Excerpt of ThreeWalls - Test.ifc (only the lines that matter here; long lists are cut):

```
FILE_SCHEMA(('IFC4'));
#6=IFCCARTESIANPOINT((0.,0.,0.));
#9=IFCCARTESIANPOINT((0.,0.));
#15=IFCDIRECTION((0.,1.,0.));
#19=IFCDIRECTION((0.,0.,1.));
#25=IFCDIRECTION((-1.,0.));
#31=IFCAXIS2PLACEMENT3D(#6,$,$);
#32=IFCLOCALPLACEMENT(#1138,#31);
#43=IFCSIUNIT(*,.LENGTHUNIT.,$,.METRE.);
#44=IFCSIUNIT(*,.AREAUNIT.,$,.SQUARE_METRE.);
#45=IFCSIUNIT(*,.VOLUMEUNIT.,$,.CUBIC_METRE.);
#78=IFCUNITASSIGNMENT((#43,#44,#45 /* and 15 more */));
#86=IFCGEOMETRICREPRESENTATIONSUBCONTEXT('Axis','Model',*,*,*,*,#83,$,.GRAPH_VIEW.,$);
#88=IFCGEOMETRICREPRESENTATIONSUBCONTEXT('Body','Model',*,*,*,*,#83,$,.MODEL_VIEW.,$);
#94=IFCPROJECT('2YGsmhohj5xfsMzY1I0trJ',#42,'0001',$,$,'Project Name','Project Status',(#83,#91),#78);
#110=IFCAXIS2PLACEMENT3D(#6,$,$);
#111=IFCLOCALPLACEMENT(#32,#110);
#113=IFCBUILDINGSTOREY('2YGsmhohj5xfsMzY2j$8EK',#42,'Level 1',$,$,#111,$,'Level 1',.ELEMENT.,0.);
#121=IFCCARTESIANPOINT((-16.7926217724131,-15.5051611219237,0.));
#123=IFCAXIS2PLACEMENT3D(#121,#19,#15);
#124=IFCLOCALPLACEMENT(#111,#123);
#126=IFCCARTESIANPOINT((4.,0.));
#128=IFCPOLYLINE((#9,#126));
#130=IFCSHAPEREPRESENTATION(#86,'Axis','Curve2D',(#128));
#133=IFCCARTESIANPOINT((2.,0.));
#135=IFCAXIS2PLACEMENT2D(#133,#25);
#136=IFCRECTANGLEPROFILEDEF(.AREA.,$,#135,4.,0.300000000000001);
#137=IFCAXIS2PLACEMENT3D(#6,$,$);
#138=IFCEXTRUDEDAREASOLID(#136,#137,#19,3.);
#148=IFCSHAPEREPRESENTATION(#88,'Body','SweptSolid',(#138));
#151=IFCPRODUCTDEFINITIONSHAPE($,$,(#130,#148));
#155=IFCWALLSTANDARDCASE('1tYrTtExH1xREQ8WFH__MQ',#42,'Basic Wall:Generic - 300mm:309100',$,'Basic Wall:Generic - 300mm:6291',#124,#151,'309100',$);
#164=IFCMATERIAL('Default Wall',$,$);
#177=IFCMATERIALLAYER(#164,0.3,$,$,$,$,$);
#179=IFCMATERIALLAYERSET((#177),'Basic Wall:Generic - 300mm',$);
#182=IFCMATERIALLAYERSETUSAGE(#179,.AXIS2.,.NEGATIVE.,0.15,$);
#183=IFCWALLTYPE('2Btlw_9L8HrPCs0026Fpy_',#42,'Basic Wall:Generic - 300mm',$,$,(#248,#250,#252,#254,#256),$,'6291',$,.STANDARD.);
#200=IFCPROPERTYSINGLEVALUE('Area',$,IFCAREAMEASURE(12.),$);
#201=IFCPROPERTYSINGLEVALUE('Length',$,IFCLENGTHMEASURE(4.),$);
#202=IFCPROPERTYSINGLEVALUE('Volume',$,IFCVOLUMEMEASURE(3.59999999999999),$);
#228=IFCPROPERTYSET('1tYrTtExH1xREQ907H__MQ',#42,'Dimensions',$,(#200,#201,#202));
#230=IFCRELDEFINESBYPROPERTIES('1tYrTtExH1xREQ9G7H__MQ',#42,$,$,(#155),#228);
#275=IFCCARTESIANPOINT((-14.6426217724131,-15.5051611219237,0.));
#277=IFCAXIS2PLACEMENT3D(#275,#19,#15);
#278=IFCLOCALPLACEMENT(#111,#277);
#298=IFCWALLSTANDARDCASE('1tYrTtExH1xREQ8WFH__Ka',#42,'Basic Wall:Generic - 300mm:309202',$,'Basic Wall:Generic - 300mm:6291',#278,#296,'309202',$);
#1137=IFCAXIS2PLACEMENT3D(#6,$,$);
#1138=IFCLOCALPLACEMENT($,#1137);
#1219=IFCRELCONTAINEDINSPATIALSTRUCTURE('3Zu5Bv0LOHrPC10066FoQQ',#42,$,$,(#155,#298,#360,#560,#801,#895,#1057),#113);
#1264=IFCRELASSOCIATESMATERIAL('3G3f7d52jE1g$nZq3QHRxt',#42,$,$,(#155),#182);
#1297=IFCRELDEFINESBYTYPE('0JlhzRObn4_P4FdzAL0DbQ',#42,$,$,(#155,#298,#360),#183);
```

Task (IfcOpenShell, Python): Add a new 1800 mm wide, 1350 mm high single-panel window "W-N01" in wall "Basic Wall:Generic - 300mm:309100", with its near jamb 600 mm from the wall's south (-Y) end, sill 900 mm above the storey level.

```python
import numpy as np
import ifcopenshell
import ifcopenshell.api.feature
import ifcopenshell.api.geometry
import ifcopenshell.api.pset
import ifcopenshell.api.root
import ifcopenshell.api.spatial
import ifcopenshell.geom
import ifcopenshell.util.element
import ifcopenshell.util.placement
import ifcopenshell.util.representation
import ifcopenshell.util.shape
import ifcopenshell.util.unit

model = ifcopenshell.open("ThreeWalls - Test.ifc")
unit_scale = ifcopenshell.util.unit.calculate_unit_scale(model)
area_scale = ifcopenshell.util.unit.calculate_unit_scale(model, "AREAUNIT")
volume_scale = ifcopenshell.util.unit.calculate_unit_scale(model, "VOLUMEUNIT")
settings = ifcopenshell.geom.settings()


def volume(element):
    """Net volume in cubic metres, openings subtracted."""
    shape = ifcopenshell.geom.create_shape(settings, element)
    return ifcopenshell.util.shape.get_volume(shape.geometry)


wall = model.by_guid("1tYrTtExH1xREQ8WFH__MQ")
storey = ifcopenshell.util.element.get_container(wall, ifc_class="IfcBuildingStorey")
context = ifcopenshell.util.representation.get_context(model, "Model", "Body", "MODEL_VIEW")
before = volume(wall)

width, height, from_end, sill = 1.8, 1.35, 0.6, 0.9  # metres

# The wall runs along its own X axis, and the end named is its -X end.
wall_shape = ifcopenshell.geom.create_shape(settings, wall)
x, y, z = ifcopenshell.util.shape.get_vertices(wall_shape.geometry).T
start = x.min() + from_end
face, thickness = float(y.min()), float(y.max() - y.min())
wall_matrix = ifcopenshell.util.placement.get_local_placement(wall.ObjectPlacement)
level = ifcopenshell.util.placement.get_local_placement(storey.ObjectPlacement)[2, 3]


def in_wall(x, y):
    """Placement at x, y metres in the wall's axes, at sill height."""
    matrix = wall_matrix.copy()
    matrix[:, 3] = wall_matrix @ np.array([x / unit_scale, y / unit_scale, 0.0, 1.0])
    matrix[2, 3] = level + sill / unit_scale
    return matrix


# Opening: a box that overshoots both wall faces by 50 mm.
opening = ifcopenshell.api.root.create_entity(model, ifc_class="IfcOpeningElement", predefined_type="OPENING")
box = ifcopenshell.api.geometry.add_wall_representation(
    model, context=context, length=width, height=height, thickness=thickness + 0.1
)
ifcopenshell.api.geometry.assign_representation(model, product=opening, representation=box)
ifcopenshell.api.geometry.edit_object_placement(model, product=opening, matrix=in_wall(start, face - 0.05), is_si=False)
ifcopenshell.api.feature.add_feature(model, feature=opening, element=wall)

window = ifcopenshell.api.root.create_entity(model, ifc_class="IfcWindow", name="W-N01", predefined_type="WINDOW")
window.OverallWidth, window.OverallHeight = width / unit_scale, height / unit_scale
window.PartitioningType = "SINGLE_PANEL"
body = ifcopenshell.api.geometry.add_window_representation(
    model,
    context=context,
    overall_width=window.OverallWidth,
    overall_height=window.OverallHeight,
    partition_type="SINGLE_PANEL",
)
ifcopenshell.api.geometry.assign_representation(model, product=window, representation=body)
ifcopenshell.api.spatial.assign_container(model, products=[window], relating_structure=storey)
ifcopenshell.api.feature.add_filling(model, opening=opening, element=window)

# Centre the window in the wall's thickness.
ifcopenshell.api.geometry.edit_object_placement(model, product=window, matrix=in_wall(start, face), is_si=False)
window_shape = ifcopenshell.geom.create_shape(settings, window)
depth = ifcopenshell.util.shape.get_vertices(window_shape.geometry)[:, 1]
offset = face + thickness / 2 - (depth.min() + depth.max()) / 2
ifcopenshell.api.geometry.edit_object_placement(model, product=window, matrix=in_wall(start, offset), is_si=False)

after = volume(wall)

# Update the wall's stored quantities.
pset = model.by_id(ifcopenshell.util.element.get_pset(wall, "Dimensions", should_inherit=False)["id"])
ifcopenshell.api.pset.edit_pset(model, pset=pset, properties={
    "Area": model.create_entity("IfcAreaMeasure", after / thickness / area_scale),
    "Volume": model.create_entity("IfcVolumeMeasure", after / volume_scale),
})

print(f"wall volume {before:.3f} -> {after:.3f} m3")

model.write("ThreeWalls - Test_rev.ifc")
```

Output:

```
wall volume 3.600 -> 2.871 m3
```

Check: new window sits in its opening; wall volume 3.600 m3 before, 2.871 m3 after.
